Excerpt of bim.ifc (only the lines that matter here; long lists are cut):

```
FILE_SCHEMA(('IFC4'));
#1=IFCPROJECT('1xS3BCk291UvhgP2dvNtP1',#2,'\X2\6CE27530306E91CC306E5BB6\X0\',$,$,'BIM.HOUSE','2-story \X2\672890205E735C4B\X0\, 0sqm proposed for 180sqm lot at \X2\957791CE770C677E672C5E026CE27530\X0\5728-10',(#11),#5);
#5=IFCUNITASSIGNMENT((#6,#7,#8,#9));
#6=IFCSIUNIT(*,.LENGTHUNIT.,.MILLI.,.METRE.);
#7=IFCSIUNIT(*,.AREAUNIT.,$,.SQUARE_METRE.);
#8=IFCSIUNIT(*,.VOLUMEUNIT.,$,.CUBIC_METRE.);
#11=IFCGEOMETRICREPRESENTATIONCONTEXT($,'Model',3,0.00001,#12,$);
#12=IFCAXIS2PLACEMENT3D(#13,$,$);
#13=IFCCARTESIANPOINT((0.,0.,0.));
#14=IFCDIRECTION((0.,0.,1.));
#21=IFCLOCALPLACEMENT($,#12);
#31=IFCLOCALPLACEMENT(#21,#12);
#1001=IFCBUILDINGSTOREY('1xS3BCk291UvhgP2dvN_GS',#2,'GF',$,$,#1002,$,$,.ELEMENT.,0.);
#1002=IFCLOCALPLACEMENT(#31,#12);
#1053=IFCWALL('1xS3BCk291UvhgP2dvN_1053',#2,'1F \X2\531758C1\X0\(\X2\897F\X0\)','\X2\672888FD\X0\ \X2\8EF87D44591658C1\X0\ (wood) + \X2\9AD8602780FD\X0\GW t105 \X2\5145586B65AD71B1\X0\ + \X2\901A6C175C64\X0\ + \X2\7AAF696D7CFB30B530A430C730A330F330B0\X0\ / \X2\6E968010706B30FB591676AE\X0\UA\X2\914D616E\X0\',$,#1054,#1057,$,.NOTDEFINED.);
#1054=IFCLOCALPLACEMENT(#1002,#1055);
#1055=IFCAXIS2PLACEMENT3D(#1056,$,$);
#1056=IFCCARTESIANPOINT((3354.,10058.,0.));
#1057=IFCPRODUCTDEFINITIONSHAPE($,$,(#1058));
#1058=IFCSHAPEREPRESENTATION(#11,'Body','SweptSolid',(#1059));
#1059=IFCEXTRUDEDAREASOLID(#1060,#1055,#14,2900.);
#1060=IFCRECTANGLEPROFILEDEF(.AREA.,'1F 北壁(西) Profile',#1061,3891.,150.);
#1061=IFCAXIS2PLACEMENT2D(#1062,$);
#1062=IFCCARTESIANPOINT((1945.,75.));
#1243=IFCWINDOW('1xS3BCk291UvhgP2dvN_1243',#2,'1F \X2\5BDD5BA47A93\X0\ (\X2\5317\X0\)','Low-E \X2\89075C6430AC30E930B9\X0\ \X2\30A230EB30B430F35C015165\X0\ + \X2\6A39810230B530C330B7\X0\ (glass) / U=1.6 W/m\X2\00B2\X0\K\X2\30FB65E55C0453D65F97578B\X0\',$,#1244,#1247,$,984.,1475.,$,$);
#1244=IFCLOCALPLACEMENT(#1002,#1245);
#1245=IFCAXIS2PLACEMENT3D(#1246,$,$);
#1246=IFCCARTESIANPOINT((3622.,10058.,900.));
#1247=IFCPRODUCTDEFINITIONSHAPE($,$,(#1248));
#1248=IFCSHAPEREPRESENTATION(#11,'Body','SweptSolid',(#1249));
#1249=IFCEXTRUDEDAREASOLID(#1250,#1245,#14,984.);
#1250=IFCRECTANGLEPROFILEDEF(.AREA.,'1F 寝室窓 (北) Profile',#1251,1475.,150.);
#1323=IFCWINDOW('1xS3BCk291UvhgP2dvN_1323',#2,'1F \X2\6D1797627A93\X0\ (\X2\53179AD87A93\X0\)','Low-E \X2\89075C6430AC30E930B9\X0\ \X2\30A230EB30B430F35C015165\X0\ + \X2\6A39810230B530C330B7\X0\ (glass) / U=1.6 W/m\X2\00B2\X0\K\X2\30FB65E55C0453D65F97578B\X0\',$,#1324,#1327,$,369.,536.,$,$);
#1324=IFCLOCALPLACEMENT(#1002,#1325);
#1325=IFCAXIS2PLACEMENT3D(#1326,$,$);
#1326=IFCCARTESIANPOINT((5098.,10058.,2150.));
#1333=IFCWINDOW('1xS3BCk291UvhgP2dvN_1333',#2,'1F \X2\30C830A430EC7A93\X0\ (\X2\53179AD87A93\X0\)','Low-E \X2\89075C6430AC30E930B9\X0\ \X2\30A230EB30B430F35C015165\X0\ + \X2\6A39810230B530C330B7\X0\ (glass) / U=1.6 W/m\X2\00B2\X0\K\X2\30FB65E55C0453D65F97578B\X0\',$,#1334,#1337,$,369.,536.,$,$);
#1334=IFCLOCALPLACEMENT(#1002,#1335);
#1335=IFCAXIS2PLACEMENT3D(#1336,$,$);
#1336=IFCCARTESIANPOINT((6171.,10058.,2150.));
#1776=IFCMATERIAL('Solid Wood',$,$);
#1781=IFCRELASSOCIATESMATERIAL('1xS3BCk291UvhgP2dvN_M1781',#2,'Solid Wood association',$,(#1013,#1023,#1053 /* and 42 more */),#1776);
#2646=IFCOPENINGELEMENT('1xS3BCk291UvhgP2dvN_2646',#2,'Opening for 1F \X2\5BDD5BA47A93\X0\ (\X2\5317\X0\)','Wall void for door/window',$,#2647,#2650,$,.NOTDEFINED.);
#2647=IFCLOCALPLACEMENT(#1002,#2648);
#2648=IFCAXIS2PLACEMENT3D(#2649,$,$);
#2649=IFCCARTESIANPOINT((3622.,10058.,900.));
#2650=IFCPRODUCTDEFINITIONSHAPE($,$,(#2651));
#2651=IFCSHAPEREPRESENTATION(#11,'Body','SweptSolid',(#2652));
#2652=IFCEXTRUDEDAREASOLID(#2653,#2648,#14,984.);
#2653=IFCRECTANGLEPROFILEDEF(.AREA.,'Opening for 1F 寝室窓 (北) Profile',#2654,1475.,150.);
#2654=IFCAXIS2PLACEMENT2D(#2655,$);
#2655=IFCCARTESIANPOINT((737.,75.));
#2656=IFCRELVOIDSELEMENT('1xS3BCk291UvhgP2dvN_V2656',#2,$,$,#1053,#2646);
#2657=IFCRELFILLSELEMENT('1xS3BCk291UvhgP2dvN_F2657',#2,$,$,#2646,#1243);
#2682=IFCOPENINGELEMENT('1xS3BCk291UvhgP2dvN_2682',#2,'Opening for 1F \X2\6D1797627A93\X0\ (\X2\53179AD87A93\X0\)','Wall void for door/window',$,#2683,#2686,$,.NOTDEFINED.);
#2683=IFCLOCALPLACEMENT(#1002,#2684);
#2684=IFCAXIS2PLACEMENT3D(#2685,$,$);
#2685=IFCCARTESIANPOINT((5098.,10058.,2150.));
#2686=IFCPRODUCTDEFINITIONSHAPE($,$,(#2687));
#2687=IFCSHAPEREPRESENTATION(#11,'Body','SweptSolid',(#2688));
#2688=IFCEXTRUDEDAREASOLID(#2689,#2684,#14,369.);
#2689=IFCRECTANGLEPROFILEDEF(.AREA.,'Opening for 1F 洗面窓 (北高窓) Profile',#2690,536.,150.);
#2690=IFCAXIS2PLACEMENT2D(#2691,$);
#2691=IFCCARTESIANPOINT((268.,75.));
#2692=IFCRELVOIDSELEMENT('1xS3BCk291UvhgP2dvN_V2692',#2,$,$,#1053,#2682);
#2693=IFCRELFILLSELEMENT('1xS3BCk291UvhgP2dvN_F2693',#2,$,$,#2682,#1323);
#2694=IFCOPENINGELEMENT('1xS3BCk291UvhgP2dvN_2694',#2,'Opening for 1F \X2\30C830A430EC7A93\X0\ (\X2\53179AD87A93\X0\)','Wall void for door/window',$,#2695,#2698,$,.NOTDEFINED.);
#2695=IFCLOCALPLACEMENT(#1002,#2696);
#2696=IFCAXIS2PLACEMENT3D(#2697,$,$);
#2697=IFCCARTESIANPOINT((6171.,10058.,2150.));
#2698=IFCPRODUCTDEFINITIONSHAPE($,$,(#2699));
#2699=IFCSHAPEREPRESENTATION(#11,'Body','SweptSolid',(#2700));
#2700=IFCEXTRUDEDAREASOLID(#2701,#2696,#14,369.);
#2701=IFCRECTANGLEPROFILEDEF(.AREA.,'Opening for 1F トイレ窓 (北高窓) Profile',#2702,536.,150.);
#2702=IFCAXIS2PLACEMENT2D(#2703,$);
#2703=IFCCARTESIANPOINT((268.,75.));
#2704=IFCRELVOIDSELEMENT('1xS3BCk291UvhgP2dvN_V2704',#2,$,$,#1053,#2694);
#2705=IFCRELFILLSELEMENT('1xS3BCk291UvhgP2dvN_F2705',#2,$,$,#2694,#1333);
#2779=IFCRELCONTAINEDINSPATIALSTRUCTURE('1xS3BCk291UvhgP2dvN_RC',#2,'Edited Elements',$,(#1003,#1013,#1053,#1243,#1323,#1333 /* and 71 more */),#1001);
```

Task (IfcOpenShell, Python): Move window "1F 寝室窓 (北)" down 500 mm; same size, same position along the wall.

```python
import numpy as np
import ifcopenshell
import ifcopenshell.api.geometry
import ifcopenshell.util.placement
import ifcopenshell.util.unit

model = ifcopenshell.open("bim.ifc")
unit_scale = ifcopenshell.util.unit.calculate_unit_scale(model)

window = model.by_guid("1xS3BCk291UvhgP2dvN_1243")
opening = window.FillsVoids[0].RelatingOpeningElement
dz = -500.0

shift = np.array([0.0, 0.0, dz])
# The window is not placed relative to its opening, so move both.
for product in (opening, window):
    matrix = ifcopenshell.util.placement.get_local_placement(product.ObjectPlacement)
    matrix[:3, 3] += shift
    ifcopenshell.api.geometry.edit_object_placement(model, product=product, matrix=matrix, is_si=False)

print(f"moved by {dz * unit_scale:+.3f} m")

model.write("bim_edited.ifc")
```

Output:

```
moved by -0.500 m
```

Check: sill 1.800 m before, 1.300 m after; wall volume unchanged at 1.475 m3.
